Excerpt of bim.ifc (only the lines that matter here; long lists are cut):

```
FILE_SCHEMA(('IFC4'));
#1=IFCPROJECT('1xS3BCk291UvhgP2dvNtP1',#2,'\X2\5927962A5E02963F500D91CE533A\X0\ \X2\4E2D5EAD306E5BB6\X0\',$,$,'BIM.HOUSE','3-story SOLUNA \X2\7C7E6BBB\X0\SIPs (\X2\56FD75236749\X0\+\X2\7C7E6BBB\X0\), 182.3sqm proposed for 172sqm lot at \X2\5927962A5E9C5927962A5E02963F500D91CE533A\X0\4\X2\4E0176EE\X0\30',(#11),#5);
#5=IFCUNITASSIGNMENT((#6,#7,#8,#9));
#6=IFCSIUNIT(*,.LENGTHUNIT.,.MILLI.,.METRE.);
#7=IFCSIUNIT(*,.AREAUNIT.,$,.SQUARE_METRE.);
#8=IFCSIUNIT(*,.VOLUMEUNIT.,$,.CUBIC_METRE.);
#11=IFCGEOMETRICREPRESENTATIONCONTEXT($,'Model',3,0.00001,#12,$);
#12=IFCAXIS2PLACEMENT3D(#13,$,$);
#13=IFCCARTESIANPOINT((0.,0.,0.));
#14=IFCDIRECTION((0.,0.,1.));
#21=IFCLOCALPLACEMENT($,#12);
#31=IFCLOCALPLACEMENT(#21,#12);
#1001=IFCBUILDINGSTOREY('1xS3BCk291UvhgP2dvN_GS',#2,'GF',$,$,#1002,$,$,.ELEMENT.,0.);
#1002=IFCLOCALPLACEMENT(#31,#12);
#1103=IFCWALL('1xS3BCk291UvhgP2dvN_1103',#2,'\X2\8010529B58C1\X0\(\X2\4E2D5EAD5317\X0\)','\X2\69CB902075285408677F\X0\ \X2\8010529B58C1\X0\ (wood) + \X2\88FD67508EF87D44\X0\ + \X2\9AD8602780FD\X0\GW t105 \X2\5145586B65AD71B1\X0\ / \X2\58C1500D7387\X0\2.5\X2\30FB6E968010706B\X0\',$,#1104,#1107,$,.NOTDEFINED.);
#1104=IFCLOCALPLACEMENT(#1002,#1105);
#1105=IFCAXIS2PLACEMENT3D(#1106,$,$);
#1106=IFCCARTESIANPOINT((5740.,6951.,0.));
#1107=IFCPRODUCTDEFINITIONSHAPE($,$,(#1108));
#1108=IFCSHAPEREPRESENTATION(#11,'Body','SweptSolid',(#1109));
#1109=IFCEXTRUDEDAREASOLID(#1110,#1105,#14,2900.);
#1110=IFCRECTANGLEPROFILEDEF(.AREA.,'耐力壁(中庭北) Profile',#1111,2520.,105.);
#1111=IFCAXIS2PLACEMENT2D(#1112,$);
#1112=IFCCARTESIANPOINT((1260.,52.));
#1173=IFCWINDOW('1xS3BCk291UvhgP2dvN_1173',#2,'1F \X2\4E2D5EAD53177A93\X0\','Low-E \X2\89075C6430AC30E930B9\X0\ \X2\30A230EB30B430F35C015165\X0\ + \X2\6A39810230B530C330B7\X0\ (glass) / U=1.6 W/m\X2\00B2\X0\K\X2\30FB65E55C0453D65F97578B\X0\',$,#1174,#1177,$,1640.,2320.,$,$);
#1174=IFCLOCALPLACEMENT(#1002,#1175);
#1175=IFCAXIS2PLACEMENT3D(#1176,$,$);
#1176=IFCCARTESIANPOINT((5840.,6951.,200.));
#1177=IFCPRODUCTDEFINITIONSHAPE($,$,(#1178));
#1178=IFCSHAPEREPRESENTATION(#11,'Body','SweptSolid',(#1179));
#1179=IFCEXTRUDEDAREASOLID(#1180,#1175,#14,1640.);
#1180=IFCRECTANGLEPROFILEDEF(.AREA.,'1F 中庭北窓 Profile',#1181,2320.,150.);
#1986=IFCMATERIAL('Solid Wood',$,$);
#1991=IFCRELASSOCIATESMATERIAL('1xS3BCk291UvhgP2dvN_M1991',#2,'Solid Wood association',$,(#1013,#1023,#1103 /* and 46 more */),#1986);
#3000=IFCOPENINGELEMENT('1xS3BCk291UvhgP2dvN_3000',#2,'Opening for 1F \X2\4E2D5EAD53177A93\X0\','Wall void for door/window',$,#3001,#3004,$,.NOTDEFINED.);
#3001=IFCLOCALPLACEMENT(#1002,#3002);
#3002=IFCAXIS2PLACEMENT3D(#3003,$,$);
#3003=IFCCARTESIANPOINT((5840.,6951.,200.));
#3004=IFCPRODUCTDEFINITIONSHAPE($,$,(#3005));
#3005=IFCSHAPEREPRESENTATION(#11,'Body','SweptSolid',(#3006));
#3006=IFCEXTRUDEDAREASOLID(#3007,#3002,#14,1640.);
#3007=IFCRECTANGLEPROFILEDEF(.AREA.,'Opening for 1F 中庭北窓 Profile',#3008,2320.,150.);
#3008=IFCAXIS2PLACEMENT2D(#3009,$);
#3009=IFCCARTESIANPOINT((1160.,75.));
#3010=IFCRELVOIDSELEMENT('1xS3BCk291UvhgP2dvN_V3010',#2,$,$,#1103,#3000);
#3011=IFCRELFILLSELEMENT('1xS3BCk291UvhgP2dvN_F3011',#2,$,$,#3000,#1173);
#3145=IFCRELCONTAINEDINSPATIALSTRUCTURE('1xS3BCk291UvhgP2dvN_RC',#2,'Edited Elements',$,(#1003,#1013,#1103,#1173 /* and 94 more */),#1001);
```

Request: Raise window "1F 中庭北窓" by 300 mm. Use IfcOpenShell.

```python
import numpy as np
import ifcopenshell
import ifcopenshell.api.geometry
import ifcopenshell.util.placement
import ifcopenshell.util.unit

model = ifcopenshell.open("bim.ifc")
unit_scale = ifcopenshell.util.unit.calculate_unit_scale(model)

window = model.by_guid("1xS3BCk291UvhgP2dvN_1173")
opening = window.FillsVoids[0].RelatingOpeningElement
dz = 0.3 / unit_scale

shift = np.array([0.0, 0.0, dz])
# The window is not placed relative to its opening, so move both.
for product in (opening, window):
    matrix = ifcopenshell.util.placement.get_local_placement(product.ObjectPlacement)
    matrix[:3, 3] += shift
    ifcopenshell.api.geometry.edit_object_placement(model, product=product, matrix=matrix, is_si=False)

print(f"moved by {dz * unit_scale:+.3f} m")

model.write("bim-out.ifc")
```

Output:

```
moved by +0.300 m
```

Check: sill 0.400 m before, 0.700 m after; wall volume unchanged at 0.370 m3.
